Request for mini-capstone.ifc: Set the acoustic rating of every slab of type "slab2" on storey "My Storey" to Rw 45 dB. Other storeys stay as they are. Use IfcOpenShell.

First a look at what the model holds.

```python
import ifcopenshell
import ifcopenshell.util.element

model = ifcopenshell.open("mini-capstone.ifc")
print(model.schema)
storey = next(s for s in model.by_type("IfcBuildingStorey") if s.Name == "My Storey")
slabs = [e for e in ifcopenshell.util.element.get_decomposition(storey) if e.is_a("IfcSlab")]
seen = {}
for e in slabs:
    element_type = ifcopenshell.util.element.get_type(e)
    key = (element_type.Name if element_type != e and element_type else None, ifcopenshell.util.element.get_pset(e, "Pset_SlabCommon", "AcousticRating"))
    seen[key] = seen.get(key, 0) + 1
for (name, value), count in sorted(seen.items(), key=str):
    print(count, "x", name, "|", value)
```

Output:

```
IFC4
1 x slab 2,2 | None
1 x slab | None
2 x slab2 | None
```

```python
import ifcopenshell
import ifcopenshell.api.pset
import ifcopenshell.util.element

model = ifcopenshell.open("mini-capstone.ifc")

storey = next(s for s in model.by_type("IfcBuildingStorey") if s.Name == "My Storey")
slabs = [e for e in ifcopenshell.util.element.get_decomposition(storey) if e.is_a("IfcSlab")]

count = 0
for e in slabs:
    element_type = ifcopenshell.util.element.get_type(e)
    if element_type in (None, e) or element_type.Name != "slab2":
        continue
    # add_pset returns the element's existing set when there is one.
    pset = ifcopenshell.api.pset.add_pset(model, product=e, name="Pset_SlabCommon")
    ifcopenshell.api.pset.edit_pset(model, pset=pset, properties={"AcousticRating": "Rw 45 dB"})
    count += 1

print(count, "slabs updated")

model.write("mini-capstone_updated.ifc")
```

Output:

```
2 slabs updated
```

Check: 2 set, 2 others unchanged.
